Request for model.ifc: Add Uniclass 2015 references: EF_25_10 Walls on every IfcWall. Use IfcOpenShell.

First a look at what the model holds.

```python
import ifcopenshell

model = ifcopenshell.open("model.ifc")
print(model.schema)
print("classifications:", [c.Name for c in model.by_type("IfcClassification")])
for ifc_class in ("IfcDoor", "IfcRoof", "IfcStair", "IfcWall", "IfcWindow"):
    print(ifc_class, len(model.by_type(ifc_class)))
```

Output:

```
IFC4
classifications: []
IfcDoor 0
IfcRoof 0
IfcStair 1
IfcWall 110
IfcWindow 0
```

```python
import ifcopenshell
import ifcopenshell.api.classification

model = ifcopenshell.open("model.ifc")

system = ifcopenshell.api.classification.add_classification(model, classification="Uniclass 2015")

codes = {
    "IfcWall": ("EF_25_10", "Walls"),
}
for ifc_class, (code, name) in codes.items():
    products = model.by_type(ifc_class)
    ifcopenshell.api.classification.add_reference(
        model, products=products, classification=system, identification=code, name=name
    )
    print(code, len(products))

model.write("model_rev.ifc")
```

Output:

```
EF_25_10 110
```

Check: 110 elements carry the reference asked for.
